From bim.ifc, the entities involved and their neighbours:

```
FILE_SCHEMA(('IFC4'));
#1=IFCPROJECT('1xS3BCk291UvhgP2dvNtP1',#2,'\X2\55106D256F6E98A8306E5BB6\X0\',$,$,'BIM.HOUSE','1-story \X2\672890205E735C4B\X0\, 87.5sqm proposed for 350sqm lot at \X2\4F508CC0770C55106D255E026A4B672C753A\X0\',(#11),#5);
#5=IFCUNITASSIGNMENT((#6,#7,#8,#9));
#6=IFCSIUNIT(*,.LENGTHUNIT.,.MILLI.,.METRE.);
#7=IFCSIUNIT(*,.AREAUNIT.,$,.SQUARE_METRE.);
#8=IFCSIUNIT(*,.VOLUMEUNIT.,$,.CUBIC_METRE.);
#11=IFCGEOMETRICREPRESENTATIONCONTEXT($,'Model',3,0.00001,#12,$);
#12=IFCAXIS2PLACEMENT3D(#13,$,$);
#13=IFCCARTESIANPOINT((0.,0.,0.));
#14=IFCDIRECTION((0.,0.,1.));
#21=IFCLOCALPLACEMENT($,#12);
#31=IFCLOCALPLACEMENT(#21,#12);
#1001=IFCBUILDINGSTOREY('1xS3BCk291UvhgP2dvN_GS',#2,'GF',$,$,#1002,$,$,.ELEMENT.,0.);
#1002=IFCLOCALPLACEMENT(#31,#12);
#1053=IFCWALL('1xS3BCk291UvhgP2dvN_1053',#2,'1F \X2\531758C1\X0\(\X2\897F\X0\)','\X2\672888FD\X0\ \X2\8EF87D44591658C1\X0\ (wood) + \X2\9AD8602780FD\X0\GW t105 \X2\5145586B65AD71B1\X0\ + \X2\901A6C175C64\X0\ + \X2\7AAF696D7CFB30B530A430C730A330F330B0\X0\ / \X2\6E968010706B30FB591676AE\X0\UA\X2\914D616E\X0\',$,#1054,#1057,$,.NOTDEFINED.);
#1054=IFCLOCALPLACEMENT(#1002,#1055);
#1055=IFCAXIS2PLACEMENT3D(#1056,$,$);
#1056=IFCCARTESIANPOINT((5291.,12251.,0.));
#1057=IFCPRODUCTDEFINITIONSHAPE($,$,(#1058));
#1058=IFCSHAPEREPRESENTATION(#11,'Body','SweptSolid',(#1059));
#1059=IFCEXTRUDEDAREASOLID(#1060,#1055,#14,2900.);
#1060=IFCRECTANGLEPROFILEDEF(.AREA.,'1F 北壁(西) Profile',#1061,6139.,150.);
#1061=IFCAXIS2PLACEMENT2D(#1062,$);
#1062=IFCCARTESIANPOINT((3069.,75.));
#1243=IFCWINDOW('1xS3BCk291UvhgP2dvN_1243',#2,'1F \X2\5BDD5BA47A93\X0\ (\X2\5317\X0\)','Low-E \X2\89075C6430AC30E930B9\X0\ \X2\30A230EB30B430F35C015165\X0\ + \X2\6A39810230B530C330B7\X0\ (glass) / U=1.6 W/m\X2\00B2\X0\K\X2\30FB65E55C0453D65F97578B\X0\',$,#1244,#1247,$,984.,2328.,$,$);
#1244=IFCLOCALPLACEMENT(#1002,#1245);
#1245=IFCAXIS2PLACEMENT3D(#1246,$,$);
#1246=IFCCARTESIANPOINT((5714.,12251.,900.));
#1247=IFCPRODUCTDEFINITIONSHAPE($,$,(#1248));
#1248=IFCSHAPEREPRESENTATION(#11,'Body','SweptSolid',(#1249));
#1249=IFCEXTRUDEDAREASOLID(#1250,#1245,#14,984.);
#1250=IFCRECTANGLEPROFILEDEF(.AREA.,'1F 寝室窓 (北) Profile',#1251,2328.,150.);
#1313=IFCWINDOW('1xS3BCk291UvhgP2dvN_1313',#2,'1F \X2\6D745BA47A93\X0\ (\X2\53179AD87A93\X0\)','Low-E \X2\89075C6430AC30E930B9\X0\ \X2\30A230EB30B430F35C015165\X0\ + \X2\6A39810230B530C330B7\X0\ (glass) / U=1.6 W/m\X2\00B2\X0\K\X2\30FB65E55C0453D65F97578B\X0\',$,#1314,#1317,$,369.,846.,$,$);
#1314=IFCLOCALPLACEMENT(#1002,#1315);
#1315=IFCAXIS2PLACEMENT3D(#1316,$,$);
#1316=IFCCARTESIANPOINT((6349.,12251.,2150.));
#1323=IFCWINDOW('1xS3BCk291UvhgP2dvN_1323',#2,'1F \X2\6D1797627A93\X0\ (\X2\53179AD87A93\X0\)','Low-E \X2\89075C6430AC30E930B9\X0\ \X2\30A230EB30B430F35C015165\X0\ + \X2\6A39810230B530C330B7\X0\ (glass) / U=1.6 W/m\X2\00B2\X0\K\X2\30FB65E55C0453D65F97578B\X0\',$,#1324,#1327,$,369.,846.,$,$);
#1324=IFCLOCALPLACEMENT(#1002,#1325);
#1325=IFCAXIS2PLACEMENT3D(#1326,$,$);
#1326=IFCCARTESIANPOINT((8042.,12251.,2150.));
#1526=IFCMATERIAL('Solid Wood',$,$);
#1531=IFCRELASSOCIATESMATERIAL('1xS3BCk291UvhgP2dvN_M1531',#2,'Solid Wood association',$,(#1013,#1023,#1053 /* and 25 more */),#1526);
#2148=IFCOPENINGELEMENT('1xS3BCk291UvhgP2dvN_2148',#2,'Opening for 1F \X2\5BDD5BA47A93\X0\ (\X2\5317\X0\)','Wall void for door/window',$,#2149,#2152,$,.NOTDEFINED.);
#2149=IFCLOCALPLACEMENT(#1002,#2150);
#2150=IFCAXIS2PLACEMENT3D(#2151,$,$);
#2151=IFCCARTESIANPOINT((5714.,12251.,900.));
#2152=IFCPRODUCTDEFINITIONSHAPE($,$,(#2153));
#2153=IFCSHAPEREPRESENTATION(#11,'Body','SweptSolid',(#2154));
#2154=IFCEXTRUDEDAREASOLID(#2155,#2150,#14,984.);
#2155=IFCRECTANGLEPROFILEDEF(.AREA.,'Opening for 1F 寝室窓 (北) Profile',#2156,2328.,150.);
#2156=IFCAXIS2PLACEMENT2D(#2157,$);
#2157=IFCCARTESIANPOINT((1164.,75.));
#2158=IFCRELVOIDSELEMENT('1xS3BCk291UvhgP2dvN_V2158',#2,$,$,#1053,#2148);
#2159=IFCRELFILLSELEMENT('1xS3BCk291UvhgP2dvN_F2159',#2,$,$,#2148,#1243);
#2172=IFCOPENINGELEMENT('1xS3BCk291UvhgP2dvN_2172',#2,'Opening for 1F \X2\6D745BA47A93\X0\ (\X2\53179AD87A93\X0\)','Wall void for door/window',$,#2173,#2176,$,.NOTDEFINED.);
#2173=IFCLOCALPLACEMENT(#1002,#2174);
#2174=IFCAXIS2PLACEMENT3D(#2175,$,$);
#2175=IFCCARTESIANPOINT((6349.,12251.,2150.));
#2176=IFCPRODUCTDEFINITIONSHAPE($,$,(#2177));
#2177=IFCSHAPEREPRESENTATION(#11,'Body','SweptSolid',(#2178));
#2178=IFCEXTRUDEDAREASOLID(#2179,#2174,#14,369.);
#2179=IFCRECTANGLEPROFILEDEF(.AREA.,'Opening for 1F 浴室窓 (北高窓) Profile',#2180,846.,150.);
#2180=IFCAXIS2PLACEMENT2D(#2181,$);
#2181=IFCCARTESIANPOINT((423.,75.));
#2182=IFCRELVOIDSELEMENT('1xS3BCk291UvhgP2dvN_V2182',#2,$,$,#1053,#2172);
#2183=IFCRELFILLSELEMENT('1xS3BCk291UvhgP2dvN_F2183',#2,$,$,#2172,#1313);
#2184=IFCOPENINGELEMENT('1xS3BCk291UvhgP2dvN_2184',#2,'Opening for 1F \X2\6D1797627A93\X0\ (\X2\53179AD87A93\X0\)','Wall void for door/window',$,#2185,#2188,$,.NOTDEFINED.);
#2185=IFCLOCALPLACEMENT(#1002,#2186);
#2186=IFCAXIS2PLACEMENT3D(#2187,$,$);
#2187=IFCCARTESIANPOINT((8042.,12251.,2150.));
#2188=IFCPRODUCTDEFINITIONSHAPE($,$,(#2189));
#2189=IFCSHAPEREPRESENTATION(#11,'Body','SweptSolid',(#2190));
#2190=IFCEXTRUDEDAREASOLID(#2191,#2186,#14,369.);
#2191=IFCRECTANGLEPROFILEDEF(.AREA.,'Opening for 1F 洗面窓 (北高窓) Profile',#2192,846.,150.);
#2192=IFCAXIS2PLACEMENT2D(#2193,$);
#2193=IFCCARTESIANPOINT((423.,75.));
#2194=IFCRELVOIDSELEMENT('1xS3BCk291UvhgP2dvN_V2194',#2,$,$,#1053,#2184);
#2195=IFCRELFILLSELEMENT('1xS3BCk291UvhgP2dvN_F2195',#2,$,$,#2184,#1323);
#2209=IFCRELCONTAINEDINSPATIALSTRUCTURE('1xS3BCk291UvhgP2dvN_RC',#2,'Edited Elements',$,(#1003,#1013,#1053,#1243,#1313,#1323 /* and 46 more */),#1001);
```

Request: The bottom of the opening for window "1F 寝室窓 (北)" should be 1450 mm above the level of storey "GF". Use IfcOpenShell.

```python
import numpy as np
import ifcopenshell
import ifcopenshell.api.geometry
import ifcopenshell.geom
import ifcopenshell.util.element
import ifcopenshell.util.placement
import ifcopenshell.util.shape
import ifcopenshell.util.unit

model = ifcopenshell.open("bim.ifc")
unit_scale = ifcopenshell.util.unit.calculate_unit_scale(model)

window = model.by_guid("1xS3BCk291UvhgP2dvN_1243")
opening = window.FillsVoids[0].RelatingOpeningElement
storey = ifcopenshell.util.element.get_container(window, ifc_class="IfcBuildingStorey")
level = ifcopenshell.util.placement.get_local_placement(storey.ObjectPlacement)[2, 3]

# The opening's origin need not be at the sill, so measure its lowest point.
shape = ifcopenshell.geom.create_shape(ifcopenshell.geom.settings(), opening)
bottom = ifcopenshell.util.shape.get_shape_bottom_elevation(shape, shape.geometry) / unit_scale
dz = level + 1.45 / unit_scale - bottom

shift = np.array([0.0, 0.0, dz])
# The window is not placed relative to its opening, so move both.
for product in (opening, window):
    matrix = ifcopenshell.util.placement.get_local_placement(product.ObjectPlacement)
    matrix[:3, 3] += shift
    ifcopenshell.api.geometry.edit_object_placement(model, product=product, matrix=matrix, is_si=False)

print(f"moved by {dz * unit_scale:+.3f} m")

model.write("bim_v2.ifc")
```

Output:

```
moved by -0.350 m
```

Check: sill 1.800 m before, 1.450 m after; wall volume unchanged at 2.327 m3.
